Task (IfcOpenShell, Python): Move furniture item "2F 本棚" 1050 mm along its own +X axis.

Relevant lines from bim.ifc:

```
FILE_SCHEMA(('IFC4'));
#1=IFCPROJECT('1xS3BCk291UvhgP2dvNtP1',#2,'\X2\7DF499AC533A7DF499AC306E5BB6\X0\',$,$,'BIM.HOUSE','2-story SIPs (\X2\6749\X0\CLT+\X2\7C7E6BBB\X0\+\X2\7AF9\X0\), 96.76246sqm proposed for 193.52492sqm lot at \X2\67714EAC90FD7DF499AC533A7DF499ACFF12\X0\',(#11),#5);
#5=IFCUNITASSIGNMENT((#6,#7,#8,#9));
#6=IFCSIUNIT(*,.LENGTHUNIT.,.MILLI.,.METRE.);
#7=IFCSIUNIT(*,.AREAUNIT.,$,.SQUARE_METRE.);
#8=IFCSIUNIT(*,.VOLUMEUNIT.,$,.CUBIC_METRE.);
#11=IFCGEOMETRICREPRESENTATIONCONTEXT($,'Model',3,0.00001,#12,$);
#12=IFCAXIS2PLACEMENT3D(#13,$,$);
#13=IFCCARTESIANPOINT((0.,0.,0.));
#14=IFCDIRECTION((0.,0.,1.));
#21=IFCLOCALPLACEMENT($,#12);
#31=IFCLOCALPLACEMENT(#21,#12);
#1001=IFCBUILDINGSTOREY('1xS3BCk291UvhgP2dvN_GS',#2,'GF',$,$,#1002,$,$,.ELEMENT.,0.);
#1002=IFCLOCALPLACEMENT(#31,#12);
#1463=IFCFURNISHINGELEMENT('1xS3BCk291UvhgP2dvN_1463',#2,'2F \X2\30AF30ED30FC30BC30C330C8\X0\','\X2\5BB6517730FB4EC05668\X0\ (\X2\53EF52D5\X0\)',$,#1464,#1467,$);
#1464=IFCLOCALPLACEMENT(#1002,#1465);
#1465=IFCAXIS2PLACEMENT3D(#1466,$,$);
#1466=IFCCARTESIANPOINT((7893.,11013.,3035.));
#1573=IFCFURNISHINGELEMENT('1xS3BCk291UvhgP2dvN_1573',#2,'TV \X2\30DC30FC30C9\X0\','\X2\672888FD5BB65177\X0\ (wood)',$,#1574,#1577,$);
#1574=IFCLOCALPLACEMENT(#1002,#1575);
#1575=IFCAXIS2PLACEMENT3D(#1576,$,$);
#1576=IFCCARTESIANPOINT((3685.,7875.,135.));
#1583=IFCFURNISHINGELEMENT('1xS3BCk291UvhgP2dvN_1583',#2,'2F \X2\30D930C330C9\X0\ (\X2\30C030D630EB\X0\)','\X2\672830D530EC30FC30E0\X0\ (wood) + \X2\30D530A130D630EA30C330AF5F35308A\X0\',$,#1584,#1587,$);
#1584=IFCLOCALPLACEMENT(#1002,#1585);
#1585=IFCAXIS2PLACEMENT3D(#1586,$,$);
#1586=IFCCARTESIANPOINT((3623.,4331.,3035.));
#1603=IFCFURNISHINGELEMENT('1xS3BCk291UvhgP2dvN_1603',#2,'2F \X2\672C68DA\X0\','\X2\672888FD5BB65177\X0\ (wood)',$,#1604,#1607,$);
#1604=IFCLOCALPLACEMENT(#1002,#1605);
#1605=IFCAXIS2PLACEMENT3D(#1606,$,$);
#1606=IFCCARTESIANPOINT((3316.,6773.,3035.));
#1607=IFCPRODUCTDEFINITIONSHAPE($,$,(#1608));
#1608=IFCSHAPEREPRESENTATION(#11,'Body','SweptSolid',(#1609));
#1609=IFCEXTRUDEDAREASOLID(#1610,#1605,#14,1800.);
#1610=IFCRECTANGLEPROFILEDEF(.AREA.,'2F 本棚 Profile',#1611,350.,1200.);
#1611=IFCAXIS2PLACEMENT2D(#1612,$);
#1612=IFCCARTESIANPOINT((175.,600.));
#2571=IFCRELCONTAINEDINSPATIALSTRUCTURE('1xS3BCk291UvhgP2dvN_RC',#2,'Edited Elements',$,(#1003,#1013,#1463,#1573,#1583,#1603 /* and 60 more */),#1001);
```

```python
import ifcopenshell
import ifcopenshell.api.geometry
import ifcopenshell.util.placement
import ifcopenshell.util.unit

model = ifcopenshell.open("bim.ifc")
unit_scale = ifcopenshell.util.unit.calculate_unit_scale(model)

item = model.by_guid("1xS3BCk291UvhgP2dvN_1603")
matrix = ifcopenshell.util.placement.get_local_placement(item.ObjectPlacement)
matrix[:3, 3] += matrix[:3, 0] * 1.05 / unit_scale
ifcopenshell.api.geometry.edit_object_placement(model, product=item, matrix=matrix, is_si=False)

print(ifcopenshell.util.placement.get_local_placement(item.ObjectPlacement).round(3) + 0.0)

model.write("bim_updated.ifc")
```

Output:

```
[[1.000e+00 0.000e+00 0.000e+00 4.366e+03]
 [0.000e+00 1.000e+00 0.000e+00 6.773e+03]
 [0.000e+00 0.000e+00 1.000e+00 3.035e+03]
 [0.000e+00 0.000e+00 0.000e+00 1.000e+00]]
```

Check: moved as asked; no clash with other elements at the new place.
